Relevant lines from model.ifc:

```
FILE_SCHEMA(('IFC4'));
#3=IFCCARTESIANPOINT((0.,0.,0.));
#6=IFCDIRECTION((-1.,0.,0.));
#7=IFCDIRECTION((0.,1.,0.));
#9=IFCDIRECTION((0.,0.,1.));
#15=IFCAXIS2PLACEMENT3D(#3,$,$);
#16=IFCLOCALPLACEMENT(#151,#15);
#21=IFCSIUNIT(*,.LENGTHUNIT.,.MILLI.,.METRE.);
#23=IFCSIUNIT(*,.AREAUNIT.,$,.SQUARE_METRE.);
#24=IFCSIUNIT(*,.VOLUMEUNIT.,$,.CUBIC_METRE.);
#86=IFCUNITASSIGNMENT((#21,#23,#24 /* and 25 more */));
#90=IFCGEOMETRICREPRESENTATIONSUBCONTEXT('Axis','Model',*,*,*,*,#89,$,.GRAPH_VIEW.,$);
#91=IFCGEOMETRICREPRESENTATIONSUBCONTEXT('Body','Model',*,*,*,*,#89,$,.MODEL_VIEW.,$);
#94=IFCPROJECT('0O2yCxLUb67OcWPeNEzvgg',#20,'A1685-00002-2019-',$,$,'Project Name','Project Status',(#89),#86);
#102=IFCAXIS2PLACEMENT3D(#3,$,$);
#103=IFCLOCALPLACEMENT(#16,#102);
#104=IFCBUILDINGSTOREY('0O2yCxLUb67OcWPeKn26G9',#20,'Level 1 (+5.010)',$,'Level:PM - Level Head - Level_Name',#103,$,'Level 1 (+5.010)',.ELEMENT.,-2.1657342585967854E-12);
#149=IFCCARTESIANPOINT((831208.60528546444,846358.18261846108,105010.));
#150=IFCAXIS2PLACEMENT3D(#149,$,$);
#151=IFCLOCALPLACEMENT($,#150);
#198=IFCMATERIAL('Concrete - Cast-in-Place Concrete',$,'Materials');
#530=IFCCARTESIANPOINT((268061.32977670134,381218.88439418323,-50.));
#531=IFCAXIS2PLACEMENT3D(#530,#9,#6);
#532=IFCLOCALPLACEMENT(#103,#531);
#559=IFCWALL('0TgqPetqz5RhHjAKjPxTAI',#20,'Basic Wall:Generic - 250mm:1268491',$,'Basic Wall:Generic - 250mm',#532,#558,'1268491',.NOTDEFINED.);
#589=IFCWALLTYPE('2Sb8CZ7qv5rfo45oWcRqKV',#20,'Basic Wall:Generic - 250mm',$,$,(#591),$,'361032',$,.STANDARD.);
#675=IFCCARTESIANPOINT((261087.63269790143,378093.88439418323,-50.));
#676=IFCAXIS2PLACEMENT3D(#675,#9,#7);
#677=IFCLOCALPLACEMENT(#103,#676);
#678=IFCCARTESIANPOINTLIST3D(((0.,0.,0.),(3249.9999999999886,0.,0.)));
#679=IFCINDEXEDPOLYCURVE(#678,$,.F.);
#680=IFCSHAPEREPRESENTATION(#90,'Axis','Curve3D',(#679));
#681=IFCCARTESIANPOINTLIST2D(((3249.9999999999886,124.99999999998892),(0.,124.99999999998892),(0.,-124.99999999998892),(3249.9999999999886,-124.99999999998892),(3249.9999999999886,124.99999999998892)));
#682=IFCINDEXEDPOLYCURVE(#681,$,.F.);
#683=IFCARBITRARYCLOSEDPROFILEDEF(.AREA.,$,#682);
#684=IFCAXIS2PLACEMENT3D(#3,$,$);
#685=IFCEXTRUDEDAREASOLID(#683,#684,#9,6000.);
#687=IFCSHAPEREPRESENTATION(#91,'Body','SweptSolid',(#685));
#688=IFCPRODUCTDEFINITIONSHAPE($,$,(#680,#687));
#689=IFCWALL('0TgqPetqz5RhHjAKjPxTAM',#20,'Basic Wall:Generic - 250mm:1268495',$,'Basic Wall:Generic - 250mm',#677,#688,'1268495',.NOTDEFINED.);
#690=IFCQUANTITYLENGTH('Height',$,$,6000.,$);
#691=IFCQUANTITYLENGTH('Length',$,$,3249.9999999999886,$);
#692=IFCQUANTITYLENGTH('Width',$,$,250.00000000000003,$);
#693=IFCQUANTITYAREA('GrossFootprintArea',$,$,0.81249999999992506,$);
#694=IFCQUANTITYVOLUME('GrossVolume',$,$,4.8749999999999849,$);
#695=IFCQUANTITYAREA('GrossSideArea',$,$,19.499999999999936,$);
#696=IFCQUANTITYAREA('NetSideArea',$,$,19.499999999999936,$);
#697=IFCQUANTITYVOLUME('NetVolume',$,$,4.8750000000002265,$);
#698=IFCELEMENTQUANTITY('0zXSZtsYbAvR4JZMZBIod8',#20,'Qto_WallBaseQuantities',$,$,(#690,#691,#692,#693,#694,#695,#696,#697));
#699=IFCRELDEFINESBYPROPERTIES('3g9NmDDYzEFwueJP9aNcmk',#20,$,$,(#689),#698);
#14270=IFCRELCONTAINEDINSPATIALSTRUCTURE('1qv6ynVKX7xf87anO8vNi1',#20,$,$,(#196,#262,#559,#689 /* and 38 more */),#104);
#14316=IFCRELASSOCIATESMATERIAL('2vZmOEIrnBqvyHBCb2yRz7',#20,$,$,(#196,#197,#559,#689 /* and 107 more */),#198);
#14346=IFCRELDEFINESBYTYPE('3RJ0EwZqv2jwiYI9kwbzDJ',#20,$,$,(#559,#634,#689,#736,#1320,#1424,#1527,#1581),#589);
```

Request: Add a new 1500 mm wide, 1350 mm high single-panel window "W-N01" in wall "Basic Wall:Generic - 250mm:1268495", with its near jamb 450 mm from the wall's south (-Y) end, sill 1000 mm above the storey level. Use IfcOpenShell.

```python
import numpy as np
import ifcopenshell
import ifcopenshell.api.feature
import ifcopenshell.api.geometry
import ifcopenshell.api.pset
import ifcopenshell.api.root
import ifcopenshell.api.spatial
import ifcopenshell.geom
import ifcopenshell.util.element
import ifcopenshell.util.placement
import ifcopenshell.util.representation
import ifcopenshell.util.shape
import ifcopenshell.util.unit

model = ifcopenshell.open("model.ifc")
unit_scale = ifcopenshell.util.unit.calculate_unit_scale(model)
area_scale = ifcopenshell.util.unit.calculate_unit_scale(model, "AREAUNIT")
volume_scale = ifcopenshell.util.unit.calculate_unit_scale(model, "VOLUMEUNIT")
settings = ifcopenshell.geom.settings()


def volume(element):
    """Net volume in cubic metres, openings subtracted."""
    shape = ifcopenshell.geom.create_shape(settings, element)
    return ifcopenshell.util.shape.get_volume(shape.geometry)


wall = model.by_guid("0TgqPetqz5RhHjAKjPxTAM")
storey = ifcopenshell.util.element.get_container(wall, ifc_class="IfcBuildingStorey")
context = ifcopenshell.util.representation.get_context(model, "Model", "Body", "MODEL_VIEW")
before = volume(wall)

width, height, from_end, sill = 1.5, 1.35, 0.45, 1  # metres

# The wall runs along its own X axis, and the end named is its -X end.
wall_shape = ifcopenshell.geom.create_shape(settings, wall)
x, y, z = ifcopenshell.util.shape.get_vertices(wall_shape.geometry).T
start = x.min() + from_end
face, thickness = float(y.min()), float(y.max() - y.min())
wall_matrix = ifcopenshell.util.placement.get_local_placement(wall.ObjectPlacement)
level = ifcopenshell.util.placement.get_local_placement(storey.ObjectPlacement)[2, 3]


def in_wall(x, y):
    """Placement at x, y metres in the wall's axes, at sill height."""
    matrix = wall_matrix.copy()
    matrix[:, 3] = wall_matrix @ np.array([x / unit_scale, y / unit_scale, 0.0, 1.0])
    matrix[2, 3] = level + sill / unit_scale
    return matrix


# Opening: a box that overshoots both wall faces by 50 mm.
opening = ifcopenshell.api.root.create_entity(model, ifc_class="IfcOpeningElement", predefined_type="OPENING")
box = ifcopenshell.api.geometry.add_wall_representation(
    model, context=context, length=width, height=height, thickness=thickness + 0.1
)
ifcopenshell.api.geometry.assign_representation(model, product=opening, representation=box)
ifcopenshell.api.geometry.edit_object_placement(model, product=opening, matrix=in_wall(start, face - 0.05), is_si=False)
ifcopenshell.api.feature.add_feature(model, feature=opening, element=wall)

window = ifcopenshell.api.root.create_entity(model, ifc_class="IfcWindow", name="W-N01", predefined_type="WINDOW")
window.OverallWidth, window.OverallHeight = width / unit_scale, height / unit_scale
window.PartitioningType = "SINGLE_PANEL"
body = ifcopenshell.api.geometry.add_window_representation(
    model,
    context=context,
    overall_width=window.OverallWidth,
    overall_height=window.OverallHeight,
    partition_type="SINGLE_PANEL",
)
ifcopenshell.api.geometry.assign_representation(model, product=window, representation=body)
ifcopenshell.api.spatial.assign_container(model, products=[window], relating_structure=storey)
ifcopenshell.api.feature.add_filling(model, opening=opening, element=window)

# Centre the window in the wall's thickness.
ifcopenshell.api.geometry.edit_object_placement(model, product=window, matrix=in_wall(start, face), is_si=False)
window_shape = ifcopenshell.geom.create_shape(settings, window)
depth = ifcopenshell.util.shape.get_vertices(window_shape.geometry)[:, 1]
offset = face + thickness / 2 - (depth.min() + depth.max()) / 2
ifcopenshell.api.geometry.edit_object_placement(model, product=window, matrix=in_wall(start, offset), is_si=False)

after = volume(wall)

# Update the wall's stored quantities.
qto = model.by_id(ifcopenshell.util.element.get_pset(wall, "Qto_WallBaseQuantities", should_inherit=False)["id"])
ifcopenshell.api.pset.edit_qto(model, qto=qto, properties={
    "NetSideArea": after / thickness / area_scale,
    "NetVolume": after / volume_scale,
})

print(f"wall volume {before:.3f} -> {after:.3f} m3")

model.write("model_v2.ifc")
```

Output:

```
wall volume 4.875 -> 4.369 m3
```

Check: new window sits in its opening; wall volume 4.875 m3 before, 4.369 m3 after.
